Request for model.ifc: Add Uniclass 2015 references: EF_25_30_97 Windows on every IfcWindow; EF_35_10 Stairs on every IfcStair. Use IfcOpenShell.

First a look at what the model holds.

```python
import ifcopenshell

model = ifcopenshell.open("model.ifc")
print(model.schema)
print("classifications:", [c.Name for c in model.by_type("IfcClassification")])
for ifc_class in ("IfcDoor", "IfcRoof", "IfcStair", "IfcWall", "IfcWindow"):
    print(ifc_class, len(model.by_type(ifc_class)))
```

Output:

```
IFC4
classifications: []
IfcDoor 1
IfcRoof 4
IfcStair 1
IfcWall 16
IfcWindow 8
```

```python
import ifcopenshell
import ifcopenshell.api.classification

model = ifcopenshell.open("model.ifc")

system = ifcopenshell.api.classification.add_classification(model, classification="Uniclass 2015")

codes = {
    "IfcWindow": ("EF_25_30_97", "Windows"),
    "IfcStair": ("EF_35_10", "Stairs"),
}
for ifc_class, (code, name) in codes.items():
    products = model.by_type(ifc_class)
    ifcopenshell.api.classification.add_reference(
        model, products=products, classification=system, identification=code, name=name
    )
    print(code, len(products))

model.write("model_edited.ifc")
```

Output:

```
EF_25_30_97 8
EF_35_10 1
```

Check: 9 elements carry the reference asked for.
